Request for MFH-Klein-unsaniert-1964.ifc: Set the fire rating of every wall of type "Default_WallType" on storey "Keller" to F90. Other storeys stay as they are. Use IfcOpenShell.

First a look at what the model holds.

```python
import ifcopenshell
import ifcopenshell.util.element

model = ifcopenshell.open("MFH-Klein-unsaniert-1964.ifc")
print(model.schema)
storey = next(s for s in model.by_type("IfcBuildingStorey") if s.Name == "Keller")
walls = [e for e in ifcopenshell.util.element.get_decomposition(storey) if e.is_a("IfcWall")]
seen = {}
for e in walls:
    element_type = ifcopenshell.util.element.get_type(e)
    key = (element_type.Name if element_type != e and element_type else None, ifcopenshell.util.element.get_pset(e, "Pset_WallCommon", "FireRating"))
    seen[key] = seen.get(key, 0) + 1
for (name, value), count in sorted(seen.items(), key=str):
    print(count, "x", name, "|", value)
```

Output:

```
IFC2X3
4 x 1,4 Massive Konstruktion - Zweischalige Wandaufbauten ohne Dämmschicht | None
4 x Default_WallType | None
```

```python
import ifcopenshell
import ifcopenshell.api.pset
import ifcopenshell.util.element

model = ifcopenshell.open("MFH-Klein-unsaniert-1964.ifc")

storey = next(s for s in model.by_type("IfcBuildingStorey") if s.Name == "Keller")
walls = [e for e in ifcopenshell.util.element.get_decomposition(storey) if e.is_a("IfcWall")]

count = 0
for e in walls:
    element_type = ifcopenshell.util.element.get_type(e)
    if element_type in (None, e) or element_type.Name != "Default_WallType":
        continue
    # add_pset returns the element's existing set when there is one.
    pset = ifcopenshell.api.pset.add_pset(model, product=e, name="Pset_WallCommon")
    ifcopenshell.api.pset.edit_pset(model, pset=pset, properties={"FireRating": "F90"})
    count += 1

print(count, "walls updated")

model.write("MFH-Klein-unsaniert-1964_updated.ifc")
```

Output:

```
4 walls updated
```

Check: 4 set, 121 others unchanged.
